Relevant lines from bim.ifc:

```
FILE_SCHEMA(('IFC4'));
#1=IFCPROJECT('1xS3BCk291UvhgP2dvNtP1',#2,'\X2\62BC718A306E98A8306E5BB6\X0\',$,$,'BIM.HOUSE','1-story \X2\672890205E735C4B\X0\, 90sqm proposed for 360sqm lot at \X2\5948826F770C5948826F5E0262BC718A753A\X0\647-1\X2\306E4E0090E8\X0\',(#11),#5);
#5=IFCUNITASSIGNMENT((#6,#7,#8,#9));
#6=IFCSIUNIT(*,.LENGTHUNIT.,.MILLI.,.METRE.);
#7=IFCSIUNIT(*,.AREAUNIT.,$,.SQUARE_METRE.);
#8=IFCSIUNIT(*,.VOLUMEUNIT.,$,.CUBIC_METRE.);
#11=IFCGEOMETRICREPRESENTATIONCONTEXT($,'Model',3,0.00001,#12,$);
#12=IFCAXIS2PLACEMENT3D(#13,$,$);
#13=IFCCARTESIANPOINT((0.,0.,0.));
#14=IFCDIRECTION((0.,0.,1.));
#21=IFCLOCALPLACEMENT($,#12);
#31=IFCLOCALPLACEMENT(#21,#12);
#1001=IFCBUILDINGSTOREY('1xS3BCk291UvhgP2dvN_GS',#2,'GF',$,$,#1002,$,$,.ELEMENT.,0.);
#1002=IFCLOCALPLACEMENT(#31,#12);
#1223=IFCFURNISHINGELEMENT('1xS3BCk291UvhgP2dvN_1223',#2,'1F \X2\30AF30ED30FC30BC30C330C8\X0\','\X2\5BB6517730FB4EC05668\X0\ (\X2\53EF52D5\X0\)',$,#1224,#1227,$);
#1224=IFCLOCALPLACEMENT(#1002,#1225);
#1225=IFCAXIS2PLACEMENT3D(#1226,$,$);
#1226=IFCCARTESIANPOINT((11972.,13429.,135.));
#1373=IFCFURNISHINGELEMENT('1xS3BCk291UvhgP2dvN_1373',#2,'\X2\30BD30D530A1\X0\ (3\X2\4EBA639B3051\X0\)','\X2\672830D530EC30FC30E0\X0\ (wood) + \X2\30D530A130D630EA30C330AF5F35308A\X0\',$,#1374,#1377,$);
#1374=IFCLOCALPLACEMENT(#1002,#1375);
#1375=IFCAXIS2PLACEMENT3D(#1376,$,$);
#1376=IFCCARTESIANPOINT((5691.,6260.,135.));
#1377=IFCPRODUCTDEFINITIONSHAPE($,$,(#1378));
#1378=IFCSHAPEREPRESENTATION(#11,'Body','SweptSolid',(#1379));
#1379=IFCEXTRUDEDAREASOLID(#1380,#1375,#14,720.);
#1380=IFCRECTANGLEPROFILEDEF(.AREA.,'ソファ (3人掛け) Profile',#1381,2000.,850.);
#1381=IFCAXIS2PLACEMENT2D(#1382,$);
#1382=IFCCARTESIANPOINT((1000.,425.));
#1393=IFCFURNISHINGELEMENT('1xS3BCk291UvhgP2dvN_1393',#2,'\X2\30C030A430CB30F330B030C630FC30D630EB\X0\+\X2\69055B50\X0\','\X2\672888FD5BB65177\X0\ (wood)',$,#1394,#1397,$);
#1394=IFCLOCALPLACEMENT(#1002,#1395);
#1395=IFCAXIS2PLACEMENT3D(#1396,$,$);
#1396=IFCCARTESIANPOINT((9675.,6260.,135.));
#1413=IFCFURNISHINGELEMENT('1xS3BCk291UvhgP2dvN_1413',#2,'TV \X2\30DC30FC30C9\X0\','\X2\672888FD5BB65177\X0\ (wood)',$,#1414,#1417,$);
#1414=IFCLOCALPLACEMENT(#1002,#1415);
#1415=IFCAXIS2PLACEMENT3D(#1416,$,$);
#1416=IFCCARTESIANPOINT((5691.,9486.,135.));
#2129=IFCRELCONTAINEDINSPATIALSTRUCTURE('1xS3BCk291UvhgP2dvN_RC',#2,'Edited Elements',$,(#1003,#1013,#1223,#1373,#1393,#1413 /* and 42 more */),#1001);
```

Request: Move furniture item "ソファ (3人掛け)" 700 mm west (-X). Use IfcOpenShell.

```python
import ifcopenshell
import ifcopenshell.api.geometry
import ifcopenshell.util.placement
import ifcopenshell.util.unit

model = ifcopenshell.open("bim.ifc")
unit_scale = ifcopenshell.util.unit.calculate_unit_scale(model)

item = model.by_guid("1xS3BCk291UvhgP2dvN_1373")
matrix = ifcopenshell.util.placement.get_local_placement(item.ObjectPlacement)
matrix[0, 3] -= 0.7 / unit_scale
ifcopenshell.api.geometry.edit_object_placement(model, product=item, matrix=matrix, is_si=False)

print(ifcopenshell.util.placement.get_local_placement(item.ObjectPlacement).round(3) + 0.0)

model.write("bim_rev.ifc")
```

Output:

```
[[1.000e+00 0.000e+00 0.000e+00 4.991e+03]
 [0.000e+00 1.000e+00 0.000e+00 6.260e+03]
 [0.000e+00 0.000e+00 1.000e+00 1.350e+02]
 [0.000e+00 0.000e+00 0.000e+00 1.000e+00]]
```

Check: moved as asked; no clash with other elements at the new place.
